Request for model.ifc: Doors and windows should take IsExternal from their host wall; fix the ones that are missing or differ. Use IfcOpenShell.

First a look at what the model holds.

```python
import ifcopenshell
import ifcopenshell.util.element

model = ifcopenshell.open("model.ifc")
print(model.schema)
seen = {}
for e in model.by_type("IfcDoor") + model.by_type("IfcWindow"):
    if not e.FillsVoids:
        continue
    host = e.FillsVoids[0].RelatingOpeningElement.VoidsElements[0].RelatingBuildingElement
    own = ifcopenshell.util.element.get_pset(e, f"Pset_{e.is_a()[3:].removesuffix('StandardCase')}Common", "IsExternal")
    wall = ifcopenshell.util.element.get_pset(host, "Pset_WallCommon", "IsExternal")
    seen[e.is_a(), own, wall] = seen.get((e.is_a(), own, wall), 0) + 1
for (cls, own, wall), count in sorted(seen.items(), key=str):
    print(count, cls, "IsExternal:", own, "| host wall:", wall)
```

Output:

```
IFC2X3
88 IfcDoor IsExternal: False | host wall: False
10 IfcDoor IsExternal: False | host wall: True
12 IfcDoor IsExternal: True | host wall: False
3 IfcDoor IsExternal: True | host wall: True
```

```python
import ifcopenshell
import ifcopenshell.api.pset
import ifcopenshell.util.element

model = ifcopenshell.open("model.ifc")

count = 0
for ifc_class, pset_name in (("IfcDoor", "Pset_DoorCommon"), ("IfcWindow", "Pset_WindowCommon")):
    for e in model.by_type(ifc_class):
        if not e.FillsVoids:
            continue
        host = e.FillsVoids[0].RelatingOpeningElement.VoidsElements[0].RelatingBuildingElement
        external = ifcopenshell.util.element.get_pset(host, "Pset_WallCommon", "IsExternal")
        if external is None or ifcopenshell.util.element.get_pset(e, pset_name, "IsExternal") == external:
            continue
        pset = ifcopenshell.api.pset.add_pset(model, product=e, name=pset_name)
        ifcopenshell.api.pset.edit_pset(model, pset=pset, properties={"IsExternal": external})
        count += 1

print(count, "updated")

model.write("model_edited.ifc")
```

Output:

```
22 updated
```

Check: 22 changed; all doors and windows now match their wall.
